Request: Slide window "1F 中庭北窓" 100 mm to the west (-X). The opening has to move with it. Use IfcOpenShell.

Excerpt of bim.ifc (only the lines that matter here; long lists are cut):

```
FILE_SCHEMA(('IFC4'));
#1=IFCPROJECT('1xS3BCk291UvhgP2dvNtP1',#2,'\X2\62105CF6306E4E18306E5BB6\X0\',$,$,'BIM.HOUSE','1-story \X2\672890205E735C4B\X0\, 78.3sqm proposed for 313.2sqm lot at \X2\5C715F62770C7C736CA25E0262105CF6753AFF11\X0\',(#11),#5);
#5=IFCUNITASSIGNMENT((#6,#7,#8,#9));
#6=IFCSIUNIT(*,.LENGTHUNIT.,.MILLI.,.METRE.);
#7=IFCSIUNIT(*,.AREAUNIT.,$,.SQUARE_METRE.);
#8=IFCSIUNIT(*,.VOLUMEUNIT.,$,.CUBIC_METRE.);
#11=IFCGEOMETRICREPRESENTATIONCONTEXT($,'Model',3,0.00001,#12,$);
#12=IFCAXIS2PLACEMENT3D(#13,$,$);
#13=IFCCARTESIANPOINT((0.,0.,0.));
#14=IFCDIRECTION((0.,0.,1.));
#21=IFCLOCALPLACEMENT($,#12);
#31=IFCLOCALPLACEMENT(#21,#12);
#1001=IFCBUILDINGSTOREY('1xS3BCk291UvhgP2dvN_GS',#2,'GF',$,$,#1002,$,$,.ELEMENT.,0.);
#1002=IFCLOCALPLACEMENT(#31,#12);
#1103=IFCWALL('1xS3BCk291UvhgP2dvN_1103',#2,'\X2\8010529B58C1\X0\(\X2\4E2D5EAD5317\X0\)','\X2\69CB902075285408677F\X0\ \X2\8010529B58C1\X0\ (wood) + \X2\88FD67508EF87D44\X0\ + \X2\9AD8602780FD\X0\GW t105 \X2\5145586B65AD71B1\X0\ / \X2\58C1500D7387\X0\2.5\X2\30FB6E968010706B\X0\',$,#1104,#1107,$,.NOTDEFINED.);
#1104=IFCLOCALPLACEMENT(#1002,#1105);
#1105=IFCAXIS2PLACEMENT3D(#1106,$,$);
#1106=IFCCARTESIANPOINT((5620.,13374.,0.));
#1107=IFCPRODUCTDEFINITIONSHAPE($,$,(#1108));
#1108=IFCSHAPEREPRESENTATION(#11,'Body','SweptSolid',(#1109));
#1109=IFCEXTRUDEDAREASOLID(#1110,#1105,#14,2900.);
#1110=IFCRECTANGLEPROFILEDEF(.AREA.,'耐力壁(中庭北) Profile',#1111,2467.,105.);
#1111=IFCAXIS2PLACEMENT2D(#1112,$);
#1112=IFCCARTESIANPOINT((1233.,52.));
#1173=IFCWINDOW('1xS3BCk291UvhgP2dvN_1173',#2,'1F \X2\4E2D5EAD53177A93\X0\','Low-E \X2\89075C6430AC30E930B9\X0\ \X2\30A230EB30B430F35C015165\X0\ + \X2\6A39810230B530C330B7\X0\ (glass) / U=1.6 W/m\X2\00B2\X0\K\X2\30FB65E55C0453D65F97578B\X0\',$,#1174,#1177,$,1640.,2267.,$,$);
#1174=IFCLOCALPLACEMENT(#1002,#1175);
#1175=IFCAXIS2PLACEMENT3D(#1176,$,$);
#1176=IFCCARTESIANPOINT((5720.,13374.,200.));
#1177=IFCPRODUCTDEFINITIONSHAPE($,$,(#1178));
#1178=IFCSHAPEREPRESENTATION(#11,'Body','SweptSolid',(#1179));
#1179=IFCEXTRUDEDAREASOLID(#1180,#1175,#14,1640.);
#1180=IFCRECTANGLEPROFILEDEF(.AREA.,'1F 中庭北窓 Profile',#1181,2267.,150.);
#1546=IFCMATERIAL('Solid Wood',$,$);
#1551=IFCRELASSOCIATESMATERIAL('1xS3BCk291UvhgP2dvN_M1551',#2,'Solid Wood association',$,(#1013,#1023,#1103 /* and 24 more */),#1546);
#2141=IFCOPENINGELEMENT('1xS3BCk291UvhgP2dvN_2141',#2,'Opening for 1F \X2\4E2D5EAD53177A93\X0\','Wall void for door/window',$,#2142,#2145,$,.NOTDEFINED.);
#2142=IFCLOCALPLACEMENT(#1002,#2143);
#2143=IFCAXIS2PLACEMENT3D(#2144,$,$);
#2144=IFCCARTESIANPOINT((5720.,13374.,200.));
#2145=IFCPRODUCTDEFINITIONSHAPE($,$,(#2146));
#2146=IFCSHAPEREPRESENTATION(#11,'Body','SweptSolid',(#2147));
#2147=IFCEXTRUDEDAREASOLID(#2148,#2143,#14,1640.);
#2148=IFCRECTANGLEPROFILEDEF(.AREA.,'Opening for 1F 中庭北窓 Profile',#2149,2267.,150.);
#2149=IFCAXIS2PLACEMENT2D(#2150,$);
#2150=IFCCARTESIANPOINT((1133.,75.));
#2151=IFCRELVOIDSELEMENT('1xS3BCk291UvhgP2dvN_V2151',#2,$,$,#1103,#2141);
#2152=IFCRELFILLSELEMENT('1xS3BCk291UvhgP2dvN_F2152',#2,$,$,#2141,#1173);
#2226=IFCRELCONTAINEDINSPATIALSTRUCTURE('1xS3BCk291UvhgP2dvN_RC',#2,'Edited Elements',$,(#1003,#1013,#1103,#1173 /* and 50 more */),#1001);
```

```python
import ifcopenshell
import ifcopenshell.api.geometry
import ifcopenshell.util.placement

model = ifcopenshell.open("bim.ifc")

window = model.by_id(1173)
opening = window.FillsVoids[0].RelatingOpeningElement
wall = opening.VoidsElements[0].RelatingBuildingElement

wall_matrix = ifcopenshell.util.placement.get_local_placement(wall.ObjectPlacement)
shift = wall_matrix[:3, 0] * -100.0
before = ifcopenshell.util.placement.get_local_placement(window.ObjectPlacement)[:3, 3].copy()

# The window is not placed relative to its opening, so move both.
for product in (opening, window):
    matrix = ifcopenshell.util.placement.get_local_placement(product.ObjectPlacement)
    matrix[:3, 3] += shift
    ifcopenshell.api.geometry.edit_object_placement(model, product=product, matrix=matrix, is_si=False)

after = ifcopenshell.util.placement.get_local_placement(window.ObjectPlacement)[:3, 3]
print("window moved by", (after - before).round(3) + 0.0)

model.write("bim_updated.ifc")
```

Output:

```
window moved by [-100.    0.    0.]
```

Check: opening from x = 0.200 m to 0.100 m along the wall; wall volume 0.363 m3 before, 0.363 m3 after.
